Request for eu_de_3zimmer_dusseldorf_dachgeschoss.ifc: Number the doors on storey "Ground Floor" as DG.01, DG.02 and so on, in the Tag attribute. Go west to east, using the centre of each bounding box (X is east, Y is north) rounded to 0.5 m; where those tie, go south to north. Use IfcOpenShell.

First a look at what the model holds.

```python
import ifcopenshell
import ifcopenshell.util.element
import ifcopenshell.util.placement

model = ifcopenshell.open("eu_de_3zimmer_dusseldorf_dachgeschoss.ifc")
print(model.schema)
storey = next(s for s in model.by_type("IfcBuildingStorey") if s.Name == "Ground Floor")
doors = [e for e in ifcopenshell.util.element.get_decomposition(storey) if e.is_a("IfcDoor")]
for e in sorted(doors, key=lambda e: e.id()):
    origin = ifcopenshell.util.placement.get_local_placement(e.ObjectPlacement)[:3, 3]
    print(e.id(), e.Tag, e.Name, origin.round(2) + 0.0, sep=" | ")
```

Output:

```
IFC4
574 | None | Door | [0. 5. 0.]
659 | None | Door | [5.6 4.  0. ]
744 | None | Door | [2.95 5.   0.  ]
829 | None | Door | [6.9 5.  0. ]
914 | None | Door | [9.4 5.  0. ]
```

```python
import ifcopenshell
import ifcopenshell.geom
import ifcopenshell.util.element
import ifcopenshell.util.shape

model = ifcopenshell.open("eu_de_3zimmer_dusseldorf_dachgeschoss.ifc")
settings = ifcopenshell.geom.settings()
settings.set("use-world-coords", True)


def centre(element):
    shape = ifcopenshell.geom.create_shape(settings, element)
    return ifcopenshell.util.shape.get_bbox_centroid(shape.geometry)


storey = next(s for s in model.by_type("IfcBuildingStorey") if s.Name == "Ground Floor")
doors = [e for e in ifcopenshell.util.element.get_decomposition(storey) if e.is_a("IfcDoor")]

# Insertion points can sit at a corner or the storey origin, so sort by the geometry (in metres).
centres = {e: centre(e) for e in doors}
doors.sort(key=lambda e: (round(centres[e][0] / 0.5), centres[e][1]))

for i, e in enumerate(doors, start=1):
    number = f"DG.{i:02d}"
    e.Tag = number
    print(e.id(), number)

model.write("eu_de_3zimmer_dusseldorf_dachgeschoss_updated.ifc")
```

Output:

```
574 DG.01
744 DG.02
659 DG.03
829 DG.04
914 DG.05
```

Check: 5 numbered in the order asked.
